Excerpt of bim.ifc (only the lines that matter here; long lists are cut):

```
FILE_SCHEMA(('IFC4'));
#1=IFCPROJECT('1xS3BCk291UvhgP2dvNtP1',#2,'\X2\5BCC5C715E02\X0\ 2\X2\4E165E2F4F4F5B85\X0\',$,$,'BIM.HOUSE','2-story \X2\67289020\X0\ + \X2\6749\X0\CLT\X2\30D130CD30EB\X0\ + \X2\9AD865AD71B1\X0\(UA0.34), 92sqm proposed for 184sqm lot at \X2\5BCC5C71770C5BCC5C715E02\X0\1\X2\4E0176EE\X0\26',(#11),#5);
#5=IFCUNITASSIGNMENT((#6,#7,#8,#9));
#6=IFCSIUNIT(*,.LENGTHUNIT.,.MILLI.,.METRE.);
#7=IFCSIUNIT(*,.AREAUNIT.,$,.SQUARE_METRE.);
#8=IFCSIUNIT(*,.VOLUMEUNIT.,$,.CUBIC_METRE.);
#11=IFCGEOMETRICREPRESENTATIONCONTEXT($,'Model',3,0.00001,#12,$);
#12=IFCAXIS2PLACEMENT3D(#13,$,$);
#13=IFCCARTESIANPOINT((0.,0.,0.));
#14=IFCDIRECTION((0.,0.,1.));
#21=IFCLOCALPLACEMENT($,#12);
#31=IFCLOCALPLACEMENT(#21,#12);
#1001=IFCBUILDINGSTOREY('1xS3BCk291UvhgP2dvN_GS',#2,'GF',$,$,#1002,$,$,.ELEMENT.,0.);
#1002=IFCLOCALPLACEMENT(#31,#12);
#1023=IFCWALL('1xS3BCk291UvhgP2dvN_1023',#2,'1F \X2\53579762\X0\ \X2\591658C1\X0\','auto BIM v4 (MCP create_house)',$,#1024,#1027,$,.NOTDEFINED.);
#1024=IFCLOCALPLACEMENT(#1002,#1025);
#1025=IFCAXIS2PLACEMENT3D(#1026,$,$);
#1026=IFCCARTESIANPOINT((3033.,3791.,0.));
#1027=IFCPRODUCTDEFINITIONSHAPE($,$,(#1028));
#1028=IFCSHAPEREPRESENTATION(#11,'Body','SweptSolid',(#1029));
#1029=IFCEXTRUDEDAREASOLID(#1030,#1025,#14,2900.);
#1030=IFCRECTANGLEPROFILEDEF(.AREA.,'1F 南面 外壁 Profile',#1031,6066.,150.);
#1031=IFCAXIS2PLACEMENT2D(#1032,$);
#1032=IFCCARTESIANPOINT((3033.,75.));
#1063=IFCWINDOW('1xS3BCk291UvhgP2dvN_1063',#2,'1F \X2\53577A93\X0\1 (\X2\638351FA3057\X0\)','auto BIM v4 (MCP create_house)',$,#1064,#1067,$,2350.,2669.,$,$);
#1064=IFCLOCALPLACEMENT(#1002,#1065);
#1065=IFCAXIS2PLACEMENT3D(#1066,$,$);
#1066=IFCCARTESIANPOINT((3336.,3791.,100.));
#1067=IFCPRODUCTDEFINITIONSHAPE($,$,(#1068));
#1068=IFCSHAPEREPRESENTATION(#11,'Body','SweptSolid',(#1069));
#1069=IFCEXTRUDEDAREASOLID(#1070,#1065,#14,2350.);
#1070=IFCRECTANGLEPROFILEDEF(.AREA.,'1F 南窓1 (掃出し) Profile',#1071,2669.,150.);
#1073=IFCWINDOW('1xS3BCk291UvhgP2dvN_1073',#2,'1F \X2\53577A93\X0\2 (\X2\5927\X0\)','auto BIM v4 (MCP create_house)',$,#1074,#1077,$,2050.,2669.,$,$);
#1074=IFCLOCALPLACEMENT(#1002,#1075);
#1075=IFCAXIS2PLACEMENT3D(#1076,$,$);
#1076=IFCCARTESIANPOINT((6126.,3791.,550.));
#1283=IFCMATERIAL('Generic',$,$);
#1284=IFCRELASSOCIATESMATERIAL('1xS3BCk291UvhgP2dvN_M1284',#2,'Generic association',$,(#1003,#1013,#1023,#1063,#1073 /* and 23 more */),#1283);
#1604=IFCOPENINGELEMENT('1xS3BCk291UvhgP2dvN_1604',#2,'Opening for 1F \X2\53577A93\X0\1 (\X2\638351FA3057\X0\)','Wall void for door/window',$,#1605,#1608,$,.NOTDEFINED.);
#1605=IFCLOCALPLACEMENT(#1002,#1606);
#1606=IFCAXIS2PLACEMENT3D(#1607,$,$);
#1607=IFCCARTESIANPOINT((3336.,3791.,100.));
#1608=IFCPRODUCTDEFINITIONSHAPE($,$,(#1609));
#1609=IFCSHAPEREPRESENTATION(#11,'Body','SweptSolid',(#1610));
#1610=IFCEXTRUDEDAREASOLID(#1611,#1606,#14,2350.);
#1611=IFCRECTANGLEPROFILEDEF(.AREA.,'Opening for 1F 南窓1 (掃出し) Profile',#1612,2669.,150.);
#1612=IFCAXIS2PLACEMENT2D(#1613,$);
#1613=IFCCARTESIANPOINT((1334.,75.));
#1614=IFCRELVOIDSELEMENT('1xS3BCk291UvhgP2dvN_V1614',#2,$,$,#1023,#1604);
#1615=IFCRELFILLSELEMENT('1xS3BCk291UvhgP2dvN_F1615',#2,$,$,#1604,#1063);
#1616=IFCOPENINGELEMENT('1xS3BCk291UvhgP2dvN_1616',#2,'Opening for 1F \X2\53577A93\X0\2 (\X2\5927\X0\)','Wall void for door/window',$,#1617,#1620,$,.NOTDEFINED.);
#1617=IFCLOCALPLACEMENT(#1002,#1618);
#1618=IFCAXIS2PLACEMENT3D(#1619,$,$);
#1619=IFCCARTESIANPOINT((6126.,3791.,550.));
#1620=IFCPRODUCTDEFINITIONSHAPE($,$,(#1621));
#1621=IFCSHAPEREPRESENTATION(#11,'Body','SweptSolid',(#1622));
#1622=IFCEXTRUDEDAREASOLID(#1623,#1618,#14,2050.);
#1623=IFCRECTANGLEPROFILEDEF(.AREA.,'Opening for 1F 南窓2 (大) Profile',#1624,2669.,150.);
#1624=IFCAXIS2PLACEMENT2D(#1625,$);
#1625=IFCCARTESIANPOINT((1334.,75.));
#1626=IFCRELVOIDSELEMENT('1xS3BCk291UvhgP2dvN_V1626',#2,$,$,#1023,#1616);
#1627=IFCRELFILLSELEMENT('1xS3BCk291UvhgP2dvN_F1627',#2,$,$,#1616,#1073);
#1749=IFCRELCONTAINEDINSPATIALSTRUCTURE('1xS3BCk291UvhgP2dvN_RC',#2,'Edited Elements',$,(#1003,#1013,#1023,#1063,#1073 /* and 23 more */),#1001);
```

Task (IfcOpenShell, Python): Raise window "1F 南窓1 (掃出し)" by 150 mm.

```python
import numpy as np
import ifcopenshell
import ifcopenshell.api.geometry
import ifcopenshell.util.placement
import ifcopenshell.util.unit

model = ifcopenshell.open("bim.ifc")
unit_scale = ifcopenshell.util.unit.calculate_unit_scale(model)

window = model.by_id(1063)
opening = window.FillsVoids[0].RelatingOpeningElement
dz = 0.15 / unit_scale

shift = np.array([0.0, 0.0, dz])
# The window is not placed relative to its opening, so move both.
for product in (opening, window):
    matrix = ifcopenshell.util.placement.get_local_placement(product.ObjectPlacement)
    matrix[:3, 3] += shift
    ifcopenshell.api.geometry.edit_object_placement(model, product=product, matrix=matrix, is_si=False)

print(f"moved by {dz * unit_scale:+.3f} m")

model.write("bim_v2.ifc")
```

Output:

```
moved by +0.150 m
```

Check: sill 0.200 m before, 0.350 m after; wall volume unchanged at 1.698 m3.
